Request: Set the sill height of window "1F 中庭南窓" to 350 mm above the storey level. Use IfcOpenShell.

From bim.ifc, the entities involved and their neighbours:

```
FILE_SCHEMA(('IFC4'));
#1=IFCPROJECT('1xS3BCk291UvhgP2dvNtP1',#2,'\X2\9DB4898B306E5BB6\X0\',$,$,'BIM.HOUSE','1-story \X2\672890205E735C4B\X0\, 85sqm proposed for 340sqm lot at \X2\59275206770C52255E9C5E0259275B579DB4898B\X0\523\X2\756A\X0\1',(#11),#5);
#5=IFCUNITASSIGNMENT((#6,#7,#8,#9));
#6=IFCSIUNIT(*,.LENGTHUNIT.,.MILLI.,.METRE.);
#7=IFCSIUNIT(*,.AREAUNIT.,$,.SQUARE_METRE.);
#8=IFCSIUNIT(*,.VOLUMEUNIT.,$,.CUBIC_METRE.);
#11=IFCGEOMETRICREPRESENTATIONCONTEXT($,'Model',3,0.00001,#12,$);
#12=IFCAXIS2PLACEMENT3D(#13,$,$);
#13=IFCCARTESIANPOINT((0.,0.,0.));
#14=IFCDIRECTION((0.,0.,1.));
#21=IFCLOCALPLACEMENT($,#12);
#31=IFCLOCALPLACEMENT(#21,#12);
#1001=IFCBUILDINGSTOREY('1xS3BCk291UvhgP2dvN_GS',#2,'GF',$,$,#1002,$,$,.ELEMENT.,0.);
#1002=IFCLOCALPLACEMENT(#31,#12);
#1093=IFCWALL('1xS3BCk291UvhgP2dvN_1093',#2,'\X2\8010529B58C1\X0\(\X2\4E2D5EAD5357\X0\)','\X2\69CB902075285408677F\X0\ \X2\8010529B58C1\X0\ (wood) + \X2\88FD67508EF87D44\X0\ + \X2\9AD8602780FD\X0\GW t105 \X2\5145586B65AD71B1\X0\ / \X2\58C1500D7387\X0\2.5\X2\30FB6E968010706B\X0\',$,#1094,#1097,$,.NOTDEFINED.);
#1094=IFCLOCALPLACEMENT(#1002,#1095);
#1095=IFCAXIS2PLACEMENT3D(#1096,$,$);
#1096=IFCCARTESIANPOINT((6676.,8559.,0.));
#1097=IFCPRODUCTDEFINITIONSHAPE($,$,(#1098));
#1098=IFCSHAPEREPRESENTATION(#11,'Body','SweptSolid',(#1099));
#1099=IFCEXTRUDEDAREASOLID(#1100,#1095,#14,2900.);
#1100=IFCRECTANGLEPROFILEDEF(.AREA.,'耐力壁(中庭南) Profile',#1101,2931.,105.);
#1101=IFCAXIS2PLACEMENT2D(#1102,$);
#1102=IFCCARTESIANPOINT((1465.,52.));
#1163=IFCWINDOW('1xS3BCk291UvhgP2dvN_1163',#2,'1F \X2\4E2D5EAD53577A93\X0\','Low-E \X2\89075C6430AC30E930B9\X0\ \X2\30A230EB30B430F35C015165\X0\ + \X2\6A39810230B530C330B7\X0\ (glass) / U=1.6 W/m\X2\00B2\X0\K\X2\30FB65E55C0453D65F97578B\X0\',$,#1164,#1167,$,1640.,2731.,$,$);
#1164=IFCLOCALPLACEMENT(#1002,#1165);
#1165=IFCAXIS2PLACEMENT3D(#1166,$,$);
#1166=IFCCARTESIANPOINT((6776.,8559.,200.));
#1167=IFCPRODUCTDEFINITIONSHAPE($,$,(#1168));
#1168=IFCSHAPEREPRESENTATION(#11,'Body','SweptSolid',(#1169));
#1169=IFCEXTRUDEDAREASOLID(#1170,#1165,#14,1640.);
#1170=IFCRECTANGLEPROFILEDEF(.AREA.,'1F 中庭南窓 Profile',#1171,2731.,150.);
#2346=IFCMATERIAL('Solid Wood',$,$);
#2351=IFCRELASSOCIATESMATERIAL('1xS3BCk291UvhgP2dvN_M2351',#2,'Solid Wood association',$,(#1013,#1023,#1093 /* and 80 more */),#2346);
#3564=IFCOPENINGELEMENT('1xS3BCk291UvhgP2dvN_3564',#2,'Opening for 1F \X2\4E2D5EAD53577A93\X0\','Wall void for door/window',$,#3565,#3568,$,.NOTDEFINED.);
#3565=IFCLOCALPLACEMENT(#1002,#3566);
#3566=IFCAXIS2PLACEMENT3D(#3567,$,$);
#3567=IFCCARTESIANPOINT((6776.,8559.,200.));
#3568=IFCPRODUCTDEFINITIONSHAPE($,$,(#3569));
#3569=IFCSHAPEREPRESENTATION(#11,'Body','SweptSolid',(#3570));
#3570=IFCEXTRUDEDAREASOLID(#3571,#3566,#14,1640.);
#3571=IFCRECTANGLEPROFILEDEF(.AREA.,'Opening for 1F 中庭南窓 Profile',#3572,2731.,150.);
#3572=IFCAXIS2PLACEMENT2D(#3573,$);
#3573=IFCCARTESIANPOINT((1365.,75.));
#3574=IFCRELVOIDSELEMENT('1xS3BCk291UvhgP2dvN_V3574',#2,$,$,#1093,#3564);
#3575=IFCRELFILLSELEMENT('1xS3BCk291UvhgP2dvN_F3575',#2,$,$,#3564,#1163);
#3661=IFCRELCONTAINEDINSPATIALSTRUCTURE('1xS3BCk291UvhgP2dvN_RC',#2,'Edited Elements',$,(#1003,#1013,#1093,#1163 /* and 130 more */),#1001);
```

```python
import numpy as np
import ifcopenshell
import ifcopenshell.api.geometry
import ifcopenshell.geom
import ifcopenshell.util.element
import ifcopenshell.util.placement
import ifcopenshell.util.shape
import ifcopenshell.util.unit

model = ifcopenshell.open("bim.ifc")
unit_scale = ifcopenshell.util.unit.calculate_unit_scale(model)

window = model.by_guid("1xS3BCk291UvhgP2dvN_1163")
opening = window.FillsVoids[0].RelatingOpeningElement
storey = ifcopenshell.util.element.get_container(window, ifc_class="IfcBuildingStorey")
level = ifcopenshell.util.placement.get_local_placement(storey.ObjectPlacement)[2, 3]

# The opening's origin need not be at the sill, so measure its lowest point.
shape = ifcopenshell.geom.create_shape(ifcopenshell.geom.settings(), opening)
bottom = ifcopenshell.util.shape.get_shape_bottom_elevation(shape, shape.geometry) / unit_scale
dz = level + 0.35 / unit_scale - bottom

shift = np.array([0.0, 0.0, dz])
# The window is not placed relative to its opening, so move both.
for product in (opening, window):
    matrix = ifcopenshell.util.placement.get_local_placement(product.ObjectPlacement)
    matrix[:3, 3] += shift
    ifcopenshell.api.geometry.edit_object_placement(model, product=product, matrix=matrix, is_si=False)

print(f"moved by {dz * unit_scale:+.3f} m")

model.write("bim_edited.ifc")
```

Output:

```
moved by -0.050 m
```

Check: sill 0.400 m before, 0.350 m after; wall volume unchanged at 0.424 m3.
